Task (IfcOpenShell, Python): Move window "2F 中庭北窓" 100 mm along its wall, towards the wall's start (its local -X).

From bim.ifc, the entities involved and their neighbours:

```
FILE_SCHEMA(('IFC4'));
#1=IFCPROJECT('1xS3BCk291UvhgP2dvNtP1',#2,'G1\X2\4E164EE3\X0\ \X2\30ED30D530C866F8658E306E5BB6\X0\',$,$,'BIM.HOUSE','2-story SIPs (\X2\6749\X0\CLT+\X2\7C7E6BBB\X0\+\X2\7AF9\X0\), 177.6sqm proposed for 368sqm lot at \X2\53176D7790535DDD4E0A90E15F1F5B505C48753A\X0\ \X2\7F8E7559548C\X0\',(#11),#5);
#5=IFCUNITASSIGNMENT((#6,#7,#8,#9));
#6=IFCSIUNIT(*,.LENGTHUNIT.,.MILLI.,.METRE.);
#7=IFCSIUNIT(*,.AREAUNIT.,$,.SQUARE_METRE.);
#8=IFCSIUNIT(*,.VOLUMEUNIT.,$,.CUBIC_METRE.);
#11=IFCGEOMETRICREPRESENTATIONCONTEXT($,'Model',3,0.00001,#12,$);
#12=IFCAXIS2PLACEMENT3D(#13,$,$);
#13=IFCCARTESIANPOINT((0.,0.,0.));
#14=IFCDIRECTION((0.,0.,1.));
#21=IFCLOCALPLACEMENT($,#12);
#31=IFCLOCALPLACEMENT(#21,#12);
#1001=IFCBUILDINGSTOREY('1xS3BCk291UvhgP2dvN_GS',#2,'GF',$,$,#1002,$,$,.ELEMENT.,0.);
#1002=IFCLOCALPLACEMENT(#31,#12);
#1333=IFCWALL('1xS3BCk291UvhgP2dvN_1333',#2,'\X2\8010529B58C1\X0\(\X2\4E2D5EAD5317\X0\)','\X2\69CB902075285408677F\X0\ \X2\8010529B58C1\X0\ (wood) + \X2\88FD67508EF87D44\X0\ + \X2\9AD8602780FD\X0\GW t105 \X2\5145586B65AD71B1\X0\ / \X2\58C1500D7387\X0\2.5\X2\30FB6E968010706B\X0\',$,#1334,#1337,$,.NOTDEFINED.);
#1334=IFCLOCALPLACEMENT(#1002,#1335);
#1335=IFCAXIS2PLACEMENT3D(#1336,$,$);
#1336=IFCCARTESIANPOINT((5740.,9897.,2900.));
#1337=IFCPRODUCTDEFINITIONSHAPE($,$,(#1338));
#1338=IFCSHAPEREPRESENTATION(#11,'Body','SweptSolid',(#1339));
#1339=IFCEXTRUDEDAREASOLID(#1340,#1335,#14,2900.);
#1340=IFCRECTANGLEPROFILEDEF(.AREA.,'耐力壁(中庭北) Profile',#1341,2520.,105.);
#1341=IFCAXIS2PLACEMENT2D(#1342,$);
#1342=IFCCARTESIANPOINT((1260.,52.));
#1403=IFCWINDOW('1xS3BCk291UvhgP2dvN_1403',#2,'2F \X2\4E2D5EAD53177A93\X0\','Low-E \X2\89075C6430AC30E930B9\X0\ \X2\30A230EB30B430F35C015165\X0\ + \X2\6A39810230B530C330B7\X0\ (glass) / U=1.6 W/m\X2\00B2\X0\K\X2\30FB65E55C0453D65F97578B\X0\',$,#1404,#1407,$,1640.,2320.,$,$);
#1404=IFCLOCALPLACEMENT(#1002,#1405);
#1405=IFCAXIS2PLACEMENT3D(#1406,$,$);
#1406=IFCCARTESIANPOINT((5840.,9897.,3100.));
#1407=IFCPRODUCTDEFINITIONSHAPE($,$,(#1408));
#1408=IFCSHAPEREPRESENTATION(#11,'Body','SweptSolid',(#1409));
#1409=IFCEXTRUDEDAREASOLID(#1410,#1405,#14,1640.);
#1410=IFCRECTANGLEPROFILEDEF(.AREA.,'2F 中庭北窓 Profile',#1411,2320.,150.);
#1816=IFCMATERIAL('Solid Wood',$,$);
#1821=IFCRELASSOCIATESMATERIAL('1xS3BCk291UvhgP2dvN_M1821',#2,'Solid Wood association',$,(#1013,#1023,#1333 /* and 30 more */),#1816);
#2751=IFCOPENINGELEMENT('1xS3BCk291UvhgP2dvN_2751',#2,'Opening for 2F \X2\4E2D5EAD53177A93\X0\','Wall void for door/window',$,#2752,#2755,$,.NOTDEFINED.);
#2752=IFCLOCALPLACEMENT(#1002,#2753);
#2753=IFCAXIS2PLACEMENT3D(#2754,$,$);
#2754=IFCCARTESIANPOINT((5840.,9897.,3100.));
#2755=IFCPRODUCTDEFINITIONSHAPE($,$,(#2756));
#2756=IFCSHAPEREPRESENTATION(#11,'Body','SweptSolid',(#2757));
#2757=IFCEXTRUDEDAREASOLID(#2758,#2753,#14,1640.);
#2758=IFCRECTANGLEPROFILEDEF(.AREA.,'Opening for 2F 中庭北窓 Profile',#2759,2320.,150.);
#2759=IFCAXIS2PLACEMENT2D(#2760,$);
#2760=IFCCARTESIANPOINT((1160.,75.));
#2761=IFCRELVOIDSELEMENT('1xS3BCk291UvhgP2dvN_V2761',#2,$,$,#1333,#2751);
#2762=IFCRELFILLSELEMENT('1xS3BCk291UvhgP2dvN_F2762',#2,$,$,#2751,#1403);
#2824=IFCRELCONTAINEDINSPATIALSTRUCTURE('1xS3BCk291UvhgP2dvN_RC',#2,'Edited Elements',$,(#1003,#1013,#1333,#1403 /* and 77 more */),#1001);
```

```python
import ifcopenshell
import ifcopenshell.api.geometry
import ifcopenshell.util.placement
import ifcopenshell.util.unit

model = ifcopenshell.open("bim.ifc")
unit_scale = ifcopenshell.util.unit.calculate_unit_scale(model)

window = model.by_guid("1xS3BCk291UvhgP2dvN_1403")
opening = window.FillsVoids[0].RelatingOpeningElement
wall = opening.VoidsElements[0].RelatingBuildingElement

wall_matrix = ifcopenshell.util.placement.get_local_placement(wall.ObjectPlacement)
shift = wall_matrix[:3, 0] * -0.1 / unit_scale
before = ifcopenshell.util.placement.get_local_placement(window.ObjectPlacement)[:3, 3].copy()

# The window is not placed relative to its opening, so move both.
for product in (opening, window):
    matrix = ifcopenshell.util.placement.get_local_placement(product.ObjectPlacement)
    matrix[:3, 3] += shift
    ifcopenshell.api.geometry.edit_object_placement(model, product=product, matrix=matrix, is_si=False)

after = ifcopenshell.util.placement.get_local_placement(window.ObjectPlacement)[:3, 3]
print("window moved by", (after - before).round(3) + 0.0)

model.write("bim-out.ifc")
```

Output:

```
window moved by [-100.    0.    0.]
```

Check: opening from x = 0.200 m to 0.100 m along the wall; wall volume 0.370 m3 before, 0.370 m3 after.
